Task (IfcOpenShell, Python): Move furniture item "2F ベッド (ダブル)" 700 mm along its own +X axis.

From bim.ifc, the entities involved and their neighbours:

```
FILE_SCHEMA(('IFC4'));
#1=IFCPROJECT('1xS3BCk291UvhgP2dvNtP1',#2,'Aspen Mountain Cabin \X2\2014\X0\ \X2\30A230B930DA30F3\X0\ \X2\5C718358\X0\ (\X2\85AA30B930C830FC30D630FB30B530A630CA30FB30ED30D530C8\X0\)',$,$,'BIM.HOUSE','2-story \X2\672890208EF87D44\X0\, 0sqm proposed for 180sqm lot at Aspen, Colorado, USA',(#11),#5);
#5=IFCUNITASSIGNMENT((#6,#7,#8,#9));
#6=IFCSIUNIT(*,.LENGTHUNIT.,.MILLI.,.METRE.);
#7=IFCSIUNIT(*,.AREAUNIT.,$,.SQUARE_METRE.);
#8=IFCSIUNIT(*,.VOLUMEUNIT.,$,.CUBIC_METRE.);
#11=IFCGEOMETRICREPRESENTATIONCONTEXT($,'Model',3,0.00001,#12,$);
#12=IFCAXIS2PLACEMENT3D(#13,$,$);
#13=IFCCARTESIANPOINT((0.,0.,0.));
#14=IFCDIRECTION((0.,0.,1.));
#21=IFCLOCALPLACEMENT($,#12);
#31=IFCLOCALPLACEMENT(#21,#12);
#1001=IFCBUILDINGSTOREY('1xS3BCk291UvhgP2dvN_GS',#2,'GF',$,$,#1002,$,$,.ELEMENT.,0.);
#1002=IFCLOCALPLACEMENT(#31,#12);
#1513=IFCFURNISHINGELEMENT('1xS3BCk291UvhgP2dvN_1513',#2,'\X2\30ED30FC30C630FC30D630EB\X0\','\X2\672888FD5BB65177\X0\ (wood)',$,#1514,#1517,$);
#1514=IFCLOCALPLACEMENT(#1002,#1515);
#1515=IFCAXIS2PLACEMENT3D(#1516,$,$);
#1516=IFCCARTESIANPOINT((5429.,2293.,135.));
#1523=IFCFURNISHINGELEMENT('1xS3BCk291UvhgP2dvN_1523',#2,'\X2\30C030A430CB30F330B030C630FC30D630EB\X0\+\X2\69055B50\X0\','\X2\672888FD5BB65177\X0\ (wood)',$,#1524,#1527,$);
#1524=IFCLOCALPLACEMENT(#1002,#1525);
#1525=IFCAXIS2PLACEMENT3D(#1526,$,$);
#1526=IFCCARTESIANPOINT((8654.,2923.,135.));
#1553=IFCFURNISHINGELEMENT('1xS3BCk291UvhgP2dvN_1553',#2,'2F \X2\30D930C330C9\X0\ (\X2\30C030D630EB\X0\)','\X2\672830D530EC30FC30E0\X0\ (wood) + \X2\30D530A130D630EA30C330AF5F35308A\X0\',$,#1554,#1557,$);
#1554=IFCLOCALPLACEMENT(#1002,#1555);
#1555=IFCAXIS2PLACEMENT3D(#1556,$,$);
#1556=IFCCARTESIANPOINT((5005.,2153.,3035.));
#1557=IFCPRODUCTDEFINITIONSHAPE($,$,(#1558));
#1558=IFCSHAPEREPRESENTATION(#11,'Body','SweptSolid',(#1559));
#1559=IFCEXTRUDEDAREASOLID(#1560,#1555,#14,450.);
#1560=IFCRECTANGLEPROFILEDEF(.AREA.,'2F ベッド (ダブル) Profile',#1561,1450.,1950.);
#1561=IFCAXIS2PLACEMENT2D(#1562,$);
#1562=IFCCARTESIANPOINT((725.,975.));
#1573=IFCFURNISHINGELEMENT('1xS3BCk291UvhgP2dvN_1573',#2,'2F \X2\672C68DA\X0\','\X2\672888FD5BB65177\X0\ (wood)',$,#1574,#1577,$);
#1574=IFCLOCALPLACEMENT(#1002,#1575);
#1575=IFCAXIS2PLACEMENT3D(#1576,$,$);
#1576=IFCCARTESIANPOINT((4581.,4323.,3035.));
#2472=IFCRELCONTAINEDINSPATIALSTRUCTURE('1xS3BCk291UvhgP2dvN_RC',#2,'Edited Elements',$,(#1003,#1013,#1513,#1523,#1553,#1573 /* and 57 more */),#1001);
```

```python
import ifcopenshell
import ifcopenshell.api.geometry
import ifcopenshell.util.placement
import ifcopenshell.util.unit

model = ifcopenshell.open("bim.ifc")
unit_scale = ifcopenshell.util.unit.calculate_unit_scale(model)

item = model.by_id(1553)
matrix = ifcopenshell.util.placement.get_local_placement(item.ObjectPlacement)
matrix[:3, 3] += matrix[:3, 0] * 0.7 / unit_scale
ifcopenshell.api.geometry.edit_object_placement(model, product=item, matrix=matrix, is_si=False)

print(ifcopenshell.util.placement.get_local_placement(item.ObjectPlacement).round(3) + 0.0)

model.write("bim-out.ifc")
```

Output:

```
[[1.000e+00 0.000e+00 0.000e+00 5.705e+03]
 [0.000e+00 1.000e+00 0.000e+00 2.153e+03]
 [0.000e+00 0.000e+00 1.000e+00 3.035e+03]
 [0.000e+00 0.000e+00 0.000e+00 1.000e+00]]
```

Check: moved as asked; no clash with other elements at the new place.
